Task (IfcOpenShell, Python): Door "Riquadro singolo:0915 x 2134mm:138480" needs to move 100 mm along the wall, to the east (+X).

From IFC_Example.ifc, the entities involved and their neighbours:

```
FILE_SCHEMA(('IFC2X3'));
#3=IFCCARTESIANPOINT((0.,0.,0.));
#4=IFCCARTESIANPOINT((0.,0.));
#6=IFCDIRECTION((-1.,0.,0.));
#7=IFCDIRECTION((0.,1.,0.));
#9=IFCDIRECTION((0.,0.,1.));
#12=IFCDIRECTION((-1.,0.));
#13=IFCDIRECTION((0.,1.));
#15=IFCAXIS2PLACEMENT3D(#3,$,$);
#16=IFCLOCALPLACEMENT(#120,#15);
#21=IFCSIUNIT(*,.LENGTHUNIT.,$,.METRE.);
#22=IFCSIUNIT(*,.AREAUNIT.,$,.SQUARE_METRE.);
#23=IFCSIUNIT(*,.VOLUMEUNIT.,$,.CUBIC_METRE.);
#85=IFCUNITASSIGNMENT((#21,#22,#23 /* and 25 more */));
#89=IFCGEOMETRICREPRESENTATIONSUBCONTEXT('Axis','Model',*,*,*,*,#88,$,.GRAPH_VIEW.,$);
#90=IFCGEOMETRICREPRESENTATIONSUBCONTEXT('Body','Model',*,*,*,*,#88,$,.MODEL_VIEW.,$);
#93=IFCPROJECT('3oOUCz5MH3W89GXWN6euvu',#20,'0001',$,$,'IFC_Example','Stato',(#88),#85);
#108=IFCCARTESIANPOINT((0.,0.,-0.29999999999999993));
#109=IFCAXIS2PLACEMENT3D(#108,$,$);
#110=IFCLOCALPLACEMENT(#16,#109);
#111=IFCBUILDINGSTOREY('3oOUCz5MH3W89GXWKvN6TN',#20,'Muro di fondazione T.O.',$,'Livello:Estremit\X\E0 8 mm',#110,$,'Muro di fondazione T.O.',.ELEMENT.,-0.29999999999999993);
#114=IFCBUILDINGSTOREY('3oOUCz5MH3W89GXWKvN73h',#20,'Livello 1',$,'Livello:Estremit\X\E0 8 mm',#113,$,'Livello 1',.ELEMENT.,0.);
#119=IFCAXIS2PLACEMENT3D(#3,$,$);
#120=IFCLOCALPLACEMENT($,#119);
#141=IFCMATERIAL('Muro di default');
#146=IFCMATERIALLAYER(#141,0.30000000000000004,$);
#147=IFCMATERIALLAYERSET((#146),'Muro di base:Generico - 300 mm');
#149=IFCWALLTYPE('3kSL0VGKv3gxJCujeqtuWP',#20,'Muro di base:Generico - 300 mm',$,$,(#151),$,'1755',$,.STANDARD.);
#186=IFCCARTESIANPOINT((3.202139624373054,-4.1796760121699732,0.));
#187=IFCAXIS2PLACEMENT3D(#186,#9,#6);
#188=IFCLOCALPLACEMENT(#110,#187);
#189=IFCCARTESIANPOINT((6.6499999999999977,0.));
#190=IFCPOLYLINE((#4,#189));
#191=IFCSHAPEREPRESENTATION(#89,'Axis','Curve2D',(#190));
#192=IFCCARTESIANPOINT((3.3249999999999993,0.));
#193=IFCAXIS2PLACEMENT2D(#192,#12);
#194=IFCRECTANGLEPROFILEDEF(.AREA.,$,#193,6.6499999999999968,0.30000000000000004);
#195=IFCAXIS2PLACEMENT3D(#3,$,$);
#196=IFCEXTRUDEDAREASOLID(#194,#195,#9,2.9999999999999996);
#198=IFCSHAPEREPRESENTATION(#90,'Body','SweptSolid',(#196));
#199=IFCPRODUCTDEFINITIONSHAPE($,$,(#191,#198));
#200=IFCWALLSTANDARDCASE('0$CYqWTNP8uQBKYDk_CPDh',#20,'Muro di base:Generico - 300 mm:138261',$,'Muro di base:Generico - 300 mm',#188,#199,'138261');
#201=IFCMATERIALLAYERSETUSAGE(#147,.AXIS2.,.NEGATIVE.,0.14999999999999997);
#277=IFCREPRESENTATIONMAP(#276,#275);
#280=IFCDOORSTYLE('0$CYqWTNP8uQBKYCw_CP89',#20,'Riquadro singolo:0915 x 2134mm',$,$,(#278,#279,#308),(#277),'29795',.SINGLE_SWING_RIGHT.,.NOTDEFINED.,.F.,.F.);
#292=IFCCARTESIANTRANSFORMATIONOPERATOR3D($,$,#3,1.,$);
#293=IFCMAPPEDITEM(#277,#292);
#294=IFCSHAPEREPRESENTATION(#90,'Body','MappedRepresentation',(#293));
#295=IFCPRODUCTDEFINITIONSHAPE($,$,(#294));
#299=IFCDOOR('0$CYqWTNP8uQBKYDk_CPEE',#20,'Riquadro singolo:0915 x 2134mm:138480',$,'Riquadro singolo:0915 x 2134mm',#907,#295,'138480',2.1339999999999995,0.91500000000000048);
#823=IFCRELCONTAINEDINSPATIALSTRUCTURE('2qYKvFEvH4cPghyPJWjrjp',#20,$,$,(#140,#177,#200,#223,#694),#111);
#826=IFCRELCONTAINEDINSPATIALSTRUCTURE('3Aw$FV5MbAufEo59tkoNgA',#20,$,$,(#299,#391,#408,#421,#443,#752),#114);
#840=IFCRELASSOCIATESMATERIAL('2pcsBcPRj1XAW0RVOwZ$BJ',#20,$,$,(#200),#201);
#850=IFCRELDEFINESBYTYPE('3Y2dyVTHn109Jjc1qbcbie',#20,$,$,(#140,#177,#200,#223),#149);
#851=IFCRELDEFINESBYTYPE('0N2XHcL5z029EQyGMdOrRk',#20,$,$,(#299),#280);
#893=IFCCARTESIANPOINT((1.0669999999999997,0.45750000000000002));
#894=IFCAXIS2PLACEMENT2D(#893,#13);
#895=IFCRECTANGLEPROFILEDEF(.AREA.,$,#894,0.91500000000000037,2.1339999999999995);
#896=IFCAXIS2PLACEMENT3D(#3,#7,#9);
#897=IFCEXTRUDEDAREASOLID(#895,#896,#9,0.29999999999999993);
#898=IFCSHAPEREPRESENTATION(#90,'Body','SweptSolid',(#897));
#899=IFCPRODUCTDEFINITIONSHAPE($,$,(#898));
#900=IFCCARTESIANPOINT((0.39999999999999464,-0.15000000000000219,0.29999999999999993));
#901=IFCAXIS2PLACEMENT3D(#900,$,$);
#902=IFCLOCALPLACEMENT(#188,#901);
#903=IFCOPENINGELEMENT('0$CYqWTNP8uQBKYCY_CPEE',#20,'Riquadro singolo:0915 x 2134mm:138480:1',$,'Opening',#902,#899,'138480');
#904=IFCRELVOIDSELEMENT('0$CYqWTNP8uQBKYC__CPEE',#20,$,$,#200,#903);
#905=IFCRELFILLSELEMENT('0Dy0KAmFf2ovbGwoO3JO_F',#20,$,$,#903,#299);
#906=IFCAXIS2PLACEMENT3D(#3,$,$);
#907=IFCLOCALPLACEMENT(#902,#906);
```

```python
import ifcopenshell
import ifcopenshell.api.geometry
import ifcopenshell.util.placement
import ifcopenshell.util.unit

model = ifcopenshell.open("IFC_Example.ifc")
unit_scale = ifcopenshell.util.unit.calculate_unit_scale(model)

door = model.by_id(299)
opening = door.FillsVoids[0].RelatingOpeningElement
wall = opening.VoidsElements[0].RelatingBuildingElement

wall_matrix = ifcopenshell.util.placement.get_local_placement(wall.ObjectPlacement)
shift = wall_matrix[:3, 0] * -0.1 / unit_scale
before = ifcopenshell.util.placement.get_local_placement(door.ObjectPlacement)[:3, 3].copy()

# The door is placed relative to its opening, so it follows when the opening moves.
matrix = ifcopenshell.util.placement.get_local_placement(opening.ObjectPlacement)
matrix[:3, 3] += shift
ifcopenshell.api.geometry.edit_object_placement(
    model, product=opening, matrix=matrix, is_si=False, should_transform_children=True
)

after = ifcopenshell.util.placement.get_local_placement(door.ObjectPlacement)[:3, 3]
print("door moved by", (after - before).round(3) + 0.0)

model.write("IFC_Example_rev.ifc")
```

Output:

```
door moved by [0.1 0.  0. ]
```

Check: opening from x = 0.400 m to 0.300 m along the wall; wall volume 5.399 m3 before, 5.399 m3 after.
